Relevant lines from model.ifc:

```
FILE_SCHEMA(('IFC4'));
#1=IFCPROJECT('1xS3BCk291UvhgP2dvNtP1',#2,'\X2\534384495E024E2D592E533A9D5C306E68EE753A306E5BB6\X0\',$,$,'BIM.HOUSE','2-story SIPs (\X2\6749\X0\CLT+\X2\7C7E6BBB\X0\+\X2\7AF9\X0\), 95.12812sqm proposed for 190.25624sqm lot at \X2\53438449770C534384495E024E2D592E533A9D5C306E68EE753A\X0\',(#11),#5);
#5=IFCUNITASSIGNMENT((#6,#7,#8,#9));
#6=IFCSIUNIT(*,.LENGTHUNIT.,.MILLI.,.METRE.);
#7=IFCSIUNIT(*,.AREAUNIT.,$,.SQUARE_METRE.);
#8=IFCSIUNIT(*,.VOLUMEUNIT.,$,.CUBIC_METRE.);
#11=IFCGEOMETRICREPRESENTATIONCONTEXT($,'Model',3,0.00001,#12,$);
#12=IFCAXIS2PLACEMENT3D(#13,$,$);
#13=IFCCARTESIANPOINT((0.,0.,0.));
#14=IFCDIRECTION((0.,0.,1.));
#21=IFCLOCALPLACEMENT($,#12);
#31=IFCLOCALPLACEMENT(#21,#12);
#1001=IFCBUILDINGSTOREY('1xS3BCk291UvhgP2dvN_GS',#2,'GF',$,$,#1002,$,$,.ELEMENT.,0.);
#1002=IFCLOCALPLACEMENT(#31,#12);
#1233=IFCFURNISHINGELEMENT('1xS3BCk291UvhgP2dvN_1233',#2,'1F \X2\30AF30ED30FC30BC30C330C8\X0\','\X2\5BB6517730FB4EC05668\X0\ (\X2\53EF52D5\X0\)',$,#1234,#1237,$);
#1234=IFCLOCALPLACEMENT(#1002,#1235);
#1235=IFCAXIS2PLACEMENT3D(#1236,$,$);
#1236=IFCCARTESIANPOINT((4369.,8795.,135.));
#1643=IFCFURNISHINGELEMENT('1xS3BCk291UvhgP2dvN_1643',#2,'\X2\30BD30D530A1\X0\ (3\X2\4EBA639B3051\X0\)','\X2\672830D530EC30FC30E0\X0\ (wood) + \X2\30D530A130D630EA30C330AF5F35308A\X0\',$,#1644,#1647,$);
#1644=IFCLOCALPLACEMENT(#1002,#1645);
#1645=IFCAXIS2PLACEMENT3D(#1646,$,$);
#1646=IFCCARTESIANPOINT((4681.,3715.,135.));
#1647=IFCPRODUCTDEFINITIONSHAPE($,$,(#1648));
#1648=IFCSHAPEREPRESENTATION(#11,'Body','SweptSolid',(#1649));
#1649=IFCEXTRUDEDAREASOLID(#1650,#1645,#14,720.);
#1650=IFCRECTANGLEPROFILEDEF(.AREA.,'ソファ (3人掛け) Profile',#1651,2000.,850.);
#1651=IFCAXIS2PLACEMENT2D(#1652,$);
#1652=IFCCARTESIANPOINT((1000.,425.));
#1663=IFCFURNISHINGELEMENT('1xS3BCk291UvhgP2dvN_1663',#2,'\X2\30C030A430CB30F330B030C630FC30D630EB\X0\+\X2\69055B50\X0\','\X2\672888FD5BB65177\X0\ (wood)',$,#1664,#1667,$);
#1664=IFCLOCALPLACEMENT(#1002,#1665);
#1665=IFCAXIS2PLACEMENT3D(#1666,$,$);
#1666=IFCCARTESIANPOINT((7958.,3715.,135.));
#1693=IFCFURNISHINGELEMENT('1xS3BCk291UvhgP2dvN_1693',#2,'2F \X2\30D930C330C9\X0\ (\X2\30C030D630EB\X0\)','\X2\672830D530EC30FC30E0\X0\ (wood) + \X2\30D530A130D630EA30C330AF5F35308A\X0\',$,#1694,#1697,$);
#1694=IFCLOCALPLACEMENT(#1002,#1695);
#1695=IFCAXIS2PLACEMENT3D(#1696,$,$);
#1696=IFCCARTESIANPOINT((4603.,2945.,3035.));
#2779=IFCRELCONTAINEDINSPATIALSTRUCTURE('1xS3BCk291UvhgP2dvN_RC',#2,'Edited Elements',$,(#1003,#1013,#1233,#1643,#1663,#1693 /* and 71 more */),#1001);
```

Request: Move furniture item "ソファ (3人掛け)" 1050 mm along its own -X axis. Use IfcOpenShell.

```python
import ifcopenshell
import ifcopenshell.api.geometry
import ifcopenshell.util.placement
import ifcopenshell.util.unit

model = ifcopenshell.open("model.ifc")
unit_scale = ifcopenshell.util.unit.calculate_unit_scale(model)

item = model.by_id(1643)
matrix = ifcopenshell.util.placement.get_local_placement(item.ObjectPlacement)
matrix[:3, 3] -= matrix[:3, 0] * 1.05 / unit_scale
ifcopenshell.api.geometry.edit_object_placement(model, product=item, matrix=matrix, is_si=False)

print(ifcopenshell.util.placement.get_local_placement(item.ObjectPlacement).round(3) + 0.0)

model.write("model_v2.ifc")
```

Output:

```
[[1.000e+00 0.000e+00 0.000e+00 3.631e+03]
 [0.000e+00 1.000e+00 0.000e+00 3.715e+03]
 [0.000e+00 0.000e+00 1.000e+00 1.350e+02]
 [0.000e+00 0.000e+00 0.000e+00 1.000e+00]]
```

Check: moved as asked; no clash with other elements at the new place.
